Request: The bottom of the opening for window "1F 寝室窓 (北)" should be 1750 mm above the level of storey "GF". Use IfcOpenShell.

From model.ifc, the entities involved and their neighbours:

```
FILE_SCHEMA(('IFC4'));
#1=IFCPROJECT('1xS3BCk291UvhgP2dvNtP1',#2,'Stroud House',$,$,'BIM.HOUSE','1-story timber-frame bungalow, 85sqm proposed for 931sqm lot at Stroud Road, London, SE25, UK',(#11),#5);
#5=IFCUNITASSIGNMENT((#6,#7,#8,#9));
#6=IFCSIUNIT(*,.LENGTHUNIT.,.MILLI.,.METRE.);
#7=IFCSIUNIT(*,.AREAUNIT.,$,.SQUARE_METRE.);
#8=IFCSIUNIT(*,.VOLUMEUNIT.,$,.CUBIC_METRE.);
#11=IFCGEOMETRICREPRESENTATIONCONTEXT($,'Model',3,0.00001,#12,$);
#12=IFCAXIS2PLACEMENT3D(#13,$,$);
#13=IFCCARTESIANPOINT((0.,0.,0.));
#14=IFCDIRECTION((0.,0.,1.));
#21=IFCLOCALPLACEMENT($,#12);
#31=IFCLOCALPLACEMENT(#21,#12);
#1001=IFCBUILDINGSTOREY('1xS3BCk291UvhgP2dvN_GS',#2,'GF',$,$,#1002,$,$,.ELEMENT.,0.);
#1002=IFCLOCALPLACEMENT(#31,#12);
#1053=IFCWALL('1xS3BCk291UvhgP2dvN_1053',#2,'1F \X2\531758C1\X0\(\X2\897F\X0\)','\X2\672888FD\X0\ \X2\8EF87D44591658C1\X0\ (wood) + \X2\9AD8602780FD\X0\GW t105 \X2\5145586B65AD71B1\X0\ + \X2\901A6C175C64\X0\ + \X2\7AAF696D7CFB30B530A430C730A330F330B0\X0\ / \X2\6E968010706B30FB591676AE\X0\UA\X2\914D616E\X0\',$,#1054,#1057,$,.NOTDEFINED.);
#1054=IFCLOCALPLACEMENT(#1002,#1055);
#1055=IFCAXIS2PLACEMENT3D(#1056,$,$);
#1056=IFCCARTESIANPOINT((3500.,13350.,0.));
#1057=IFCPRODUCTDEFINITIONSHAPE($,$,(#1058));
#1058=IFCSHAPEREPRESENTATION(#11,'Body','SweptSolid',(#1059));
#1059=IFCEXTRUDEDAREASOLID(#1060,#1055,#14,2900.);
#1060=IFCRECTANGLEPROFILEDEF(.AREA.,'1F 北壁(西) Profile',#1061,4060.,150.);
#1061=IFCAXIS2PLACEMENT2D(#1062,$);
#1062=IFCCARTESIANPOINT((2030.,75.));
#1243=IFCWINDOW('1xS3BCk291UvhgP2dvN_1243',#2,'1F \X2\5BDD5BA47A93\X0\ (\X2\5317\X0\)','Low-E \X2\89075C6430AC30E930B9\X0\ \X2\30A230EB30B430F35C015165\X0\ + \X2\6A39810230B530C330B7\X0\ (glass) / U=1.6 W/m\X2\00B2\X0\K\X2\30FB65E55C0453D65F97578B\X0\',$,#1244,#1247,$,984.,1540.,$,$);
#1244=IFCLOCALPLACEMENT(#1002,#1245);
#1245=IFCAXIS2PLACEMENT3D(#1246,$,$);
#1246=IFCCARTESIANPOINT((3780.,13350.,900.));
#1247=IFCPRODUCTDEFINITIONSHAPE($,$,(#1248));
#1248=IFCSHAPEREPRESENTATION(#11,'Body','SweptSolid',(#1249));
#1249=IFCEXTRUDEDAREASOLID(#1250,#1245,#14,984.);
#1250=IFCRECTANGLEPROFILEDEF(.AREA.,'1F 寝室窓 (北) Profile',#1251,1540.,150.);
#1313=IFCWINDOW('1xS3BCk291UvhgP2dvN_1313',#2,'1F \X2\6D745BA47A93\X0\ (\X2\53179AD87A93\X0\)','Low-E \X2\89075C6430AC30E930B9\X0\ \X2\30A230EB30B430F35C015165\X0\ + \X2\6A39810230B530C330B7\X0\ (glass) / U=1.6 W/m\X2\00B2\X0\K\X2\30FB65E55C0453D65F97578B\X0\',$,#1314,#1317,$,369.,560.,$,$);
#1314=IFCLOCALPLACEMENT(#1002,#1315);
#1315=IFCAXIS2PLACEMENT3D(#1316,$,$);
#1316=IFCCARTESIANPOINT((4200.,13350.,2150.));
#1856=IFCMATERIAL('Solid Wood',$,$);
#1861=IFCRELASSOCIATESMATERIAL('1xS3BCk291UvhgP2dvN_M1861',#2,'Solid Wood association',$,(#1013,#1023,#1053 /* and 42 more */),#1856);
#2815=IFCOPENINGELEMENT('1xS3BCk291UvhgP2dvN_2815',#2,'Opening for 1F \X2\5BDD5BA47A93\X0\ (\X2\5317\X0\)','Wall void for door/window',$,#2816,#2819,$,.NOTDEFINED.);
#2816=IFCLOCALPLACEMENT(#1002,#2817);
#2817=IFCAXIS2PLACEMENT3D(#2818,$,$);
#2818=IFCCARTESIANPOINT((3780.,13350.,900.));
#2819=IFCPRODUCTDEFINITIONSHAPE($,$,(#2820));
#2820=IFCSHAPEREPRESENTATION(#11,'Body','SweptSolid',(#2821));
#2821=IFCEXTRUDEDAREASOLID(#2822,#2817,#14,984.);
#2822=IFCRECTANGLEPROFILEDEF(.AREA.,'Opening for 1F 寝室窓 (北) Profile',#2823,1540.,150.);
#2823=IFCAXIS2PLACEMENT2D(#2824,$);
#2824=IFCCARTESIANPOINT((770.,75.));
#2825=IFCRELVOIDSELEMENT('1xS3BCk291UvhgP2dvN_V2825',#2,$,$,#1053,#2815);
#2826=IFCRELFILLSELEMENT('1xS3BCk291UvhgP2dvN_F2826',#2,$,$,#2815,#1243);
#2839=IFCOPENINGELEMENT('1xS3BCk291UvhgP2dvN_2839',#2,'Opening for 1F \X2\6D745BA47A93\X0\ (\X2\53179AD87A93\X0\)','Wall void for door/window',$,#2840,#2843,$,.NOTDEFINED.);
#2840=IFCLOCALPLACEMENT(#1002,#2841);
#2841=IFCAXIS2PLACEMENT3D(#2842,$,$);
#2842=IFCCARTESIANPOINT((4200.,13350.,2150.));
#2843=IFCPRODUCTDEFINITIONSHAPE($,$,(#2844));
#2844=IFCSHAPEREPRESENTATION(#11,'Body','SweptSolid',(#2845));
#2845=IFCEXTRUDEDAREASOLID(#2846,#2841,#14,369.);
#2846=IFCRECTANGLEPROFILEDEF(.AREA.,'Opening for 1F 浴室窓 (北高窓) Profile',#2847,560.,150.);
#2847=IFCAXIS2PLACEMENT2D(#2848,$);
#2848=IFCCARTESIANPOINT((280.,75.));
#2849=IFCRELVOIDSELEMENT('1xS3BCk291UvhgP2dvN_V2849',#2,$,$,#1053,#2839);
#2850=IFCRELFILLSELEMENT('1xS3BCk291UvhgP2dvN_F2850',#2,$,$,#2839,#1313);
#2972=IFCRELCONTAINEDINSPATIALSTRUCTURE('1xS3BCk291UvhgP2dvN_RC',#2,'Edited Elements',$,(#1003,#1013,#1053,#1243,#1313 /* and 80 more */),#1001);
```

```python
import numpy as np
import ifcopenshell
import ifcopenshell.api.geometry
import ifcopenshell.geom
import ifcopenshell.util.element
import ifcopenshell.util.placement
import ifcopenshell.util.shape
import ifcopenshell.util.unit

model = ifcopenshell.open("model.ifc")
unit_scale = ifcopenshell.util.unit.calculate_unit_scale(model)

window = model.by_id(1243)
opening = window.FillsVoids[0].RelatingOpeningElement
storey = ifcopenshell.util.element.get_container(window, ifc_class="IfcBuildingStorey")
level = ifcopenshell.util.placement.get_local_placement(storey.ObjectPlacement)[2, 3]

# The opening's origin need not be at the sill, so measure its lowest point.
shape = ifcopenshell.geom.create_shape(ifcopenshell.geom.settings(), opening)
bottom = ifcopenshell.util.shape.get_shape_bottom_elevation(shape, shape.geometry) / unit_scale
dz = level + 1.75 / unit_scale - bottom

shift = np.array([0.0, 0.0, dz])
# The window is not placed relative to its opening, so move both.
for product in (opening, window):
    matrix = ifcopenshell.util.placement.get_local_placement(product.ObjectPlacement)
    matrix[:3, 3] += shift
    ifcopenshell.api.geometry.edit_object_placement(model, product=product, matrix=matrix, is_si=False)

print(f"moved by {dz * unit_scale:+.3f} m")

model.write("model-out.ifc")
```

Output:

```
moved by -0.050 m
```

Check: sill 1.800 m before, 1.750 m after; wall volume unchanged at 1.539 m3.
